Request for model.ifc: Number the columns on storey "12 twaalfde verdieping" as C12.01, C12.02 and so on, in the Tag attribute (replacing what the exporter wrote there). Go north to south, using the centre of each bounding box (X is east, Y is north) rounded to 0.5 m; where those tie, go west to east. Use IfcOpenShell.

First a look at what the model holds.

```python
import ifcopenshell
import ifcopenshell.util.element
import ifcopenshell.util.placement

model = ifcopenshell.open("model.ifc")
print(model.schema)
storey = next(s for s in model.by_type("IfcBuildingStorey") if s.Name == "12 twaalfde verdieping")
columns = [e for e in ifcopenshell.util.element.get_decomposition(storey) if e.is_a("IfcColumn")]
for e in sorted(columns, key=lambda e: e.id()):
    origin = ifcopenshell.util.placement.get_local_placement(e.ObjectPlacement)[:3, 3]
    print(e.id(), e.Tag, e.Name, origin.round(2) + 0.0, sep=" | ")
```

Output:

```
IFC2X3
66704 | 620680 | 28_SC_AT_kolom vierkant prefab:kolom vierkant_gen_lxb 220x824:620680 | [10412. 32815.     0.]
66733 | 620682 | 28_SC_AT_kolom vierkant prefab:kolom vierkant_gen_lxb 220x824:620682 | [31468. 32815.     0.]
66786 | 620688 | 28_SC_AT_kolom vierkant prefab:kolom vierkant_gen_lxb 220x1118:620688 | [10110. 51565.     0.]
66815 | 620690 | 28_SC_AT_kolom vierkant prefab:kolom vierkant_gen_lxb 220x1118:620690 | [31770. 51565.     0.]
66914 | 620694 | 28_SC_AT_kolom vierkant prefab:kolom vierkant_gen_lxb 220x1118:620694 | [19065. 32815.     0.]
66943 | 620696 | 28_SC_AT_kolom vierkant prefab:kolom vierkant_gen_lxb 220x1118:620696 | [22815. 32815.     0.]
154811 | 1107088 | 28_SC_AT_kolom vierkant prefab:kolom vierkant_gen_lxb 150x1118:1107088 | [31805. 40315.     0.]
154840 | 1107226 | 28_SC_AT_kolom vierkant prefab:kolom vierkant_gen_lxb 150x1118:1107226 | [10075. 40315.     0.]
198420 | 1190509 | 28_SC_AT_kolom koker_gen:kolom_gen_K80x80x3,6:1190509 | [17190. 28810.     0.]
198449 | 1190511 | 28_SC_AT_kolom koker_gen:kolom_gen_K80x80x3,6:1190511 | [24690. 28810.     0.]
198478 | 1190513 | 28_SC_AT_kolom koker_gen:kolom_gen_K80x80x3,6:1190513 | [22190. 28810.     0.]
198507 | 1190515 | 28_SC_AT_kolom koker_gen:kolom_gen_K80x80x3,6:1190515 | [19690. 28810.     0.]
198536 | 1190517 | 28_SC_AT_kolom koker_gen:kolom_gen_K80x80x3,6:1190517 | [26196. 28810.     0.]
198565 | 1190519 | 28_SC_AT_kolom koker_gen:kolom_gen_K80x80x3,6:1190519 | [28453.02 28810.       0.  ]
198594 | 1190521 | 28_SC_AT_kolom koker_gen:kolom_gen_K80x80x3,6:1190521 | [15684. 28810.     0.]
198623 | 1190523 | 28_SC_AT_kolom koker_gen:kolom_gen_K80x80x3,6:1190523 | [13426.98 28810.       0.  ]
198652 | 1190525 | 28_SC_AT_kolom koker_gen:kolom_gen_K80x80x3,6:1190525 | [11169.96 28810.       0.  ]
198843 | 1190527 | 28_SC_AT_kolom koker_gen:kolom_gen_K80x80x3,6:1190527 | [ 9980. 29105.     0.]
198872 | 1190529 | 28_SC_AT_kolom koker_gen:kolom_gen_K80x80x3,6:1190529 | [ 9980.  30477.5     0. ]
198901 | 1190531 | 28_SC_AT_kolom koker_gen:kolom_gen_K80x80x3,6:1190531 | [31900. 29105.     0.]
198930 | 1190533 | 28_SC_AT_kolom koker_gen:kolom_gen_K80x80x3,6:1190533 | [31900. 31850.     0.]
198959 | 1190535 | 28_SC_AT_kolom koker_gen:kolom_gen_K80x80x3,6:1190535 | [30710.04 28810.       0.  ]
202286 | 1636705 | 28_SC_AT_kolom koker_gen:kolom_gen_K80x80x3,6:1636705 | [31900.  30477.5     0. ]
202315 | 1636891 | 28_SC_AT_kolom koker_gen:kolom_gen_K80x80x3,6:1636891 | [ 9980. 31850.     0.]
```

```python
import ifcopenshell
import ifcopenshell.geom
import ifcopenshell.util.element
import ifcopenshell.util.shape

model = ifcopenshell.open("model.ifc")
settings = ifcopenshell.geom.settings()
settings.set("use-world-coords", True)


def centre(element):
    shape = ifcopenshell.geom.create_shape(settings, element)
    return ifcopenshell.util.shape.get_bbox_centroid(shape.geometry)


storey = next(s for s in model.by_type("IfcBuildingStorey") if s.Name == "12 twaalfde verdieping")
columns = [e for e in ifcopenshell.util.element.get_decomposition(storey) if e.is_a("IfcColumn")]

# Insertion points can sit at a corner or the storey origin, so sort by the geometry (in metres).
centres = {e: centre(e) for e in columns}
columns.sort(key=lambda e: (-round(centres[e][1] / 0.5), centres[e][0]))

for i, e in enumerate(columns, start=1):
    number = f"C12.{i:02d}"
    e.Tag = number
    print(e.id(), number)

model.write("model-out.ifc")
```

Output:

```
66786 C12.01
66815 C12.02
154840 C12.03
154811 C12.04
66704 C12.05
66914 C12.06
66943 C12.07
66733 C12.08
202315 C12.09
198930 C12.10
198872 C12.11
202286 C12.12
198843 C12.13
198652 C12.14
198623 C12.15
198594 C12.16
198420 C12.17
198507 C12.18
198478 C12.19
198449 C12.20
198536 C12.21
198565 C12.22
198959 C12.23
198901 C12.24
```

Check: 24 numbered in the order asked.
